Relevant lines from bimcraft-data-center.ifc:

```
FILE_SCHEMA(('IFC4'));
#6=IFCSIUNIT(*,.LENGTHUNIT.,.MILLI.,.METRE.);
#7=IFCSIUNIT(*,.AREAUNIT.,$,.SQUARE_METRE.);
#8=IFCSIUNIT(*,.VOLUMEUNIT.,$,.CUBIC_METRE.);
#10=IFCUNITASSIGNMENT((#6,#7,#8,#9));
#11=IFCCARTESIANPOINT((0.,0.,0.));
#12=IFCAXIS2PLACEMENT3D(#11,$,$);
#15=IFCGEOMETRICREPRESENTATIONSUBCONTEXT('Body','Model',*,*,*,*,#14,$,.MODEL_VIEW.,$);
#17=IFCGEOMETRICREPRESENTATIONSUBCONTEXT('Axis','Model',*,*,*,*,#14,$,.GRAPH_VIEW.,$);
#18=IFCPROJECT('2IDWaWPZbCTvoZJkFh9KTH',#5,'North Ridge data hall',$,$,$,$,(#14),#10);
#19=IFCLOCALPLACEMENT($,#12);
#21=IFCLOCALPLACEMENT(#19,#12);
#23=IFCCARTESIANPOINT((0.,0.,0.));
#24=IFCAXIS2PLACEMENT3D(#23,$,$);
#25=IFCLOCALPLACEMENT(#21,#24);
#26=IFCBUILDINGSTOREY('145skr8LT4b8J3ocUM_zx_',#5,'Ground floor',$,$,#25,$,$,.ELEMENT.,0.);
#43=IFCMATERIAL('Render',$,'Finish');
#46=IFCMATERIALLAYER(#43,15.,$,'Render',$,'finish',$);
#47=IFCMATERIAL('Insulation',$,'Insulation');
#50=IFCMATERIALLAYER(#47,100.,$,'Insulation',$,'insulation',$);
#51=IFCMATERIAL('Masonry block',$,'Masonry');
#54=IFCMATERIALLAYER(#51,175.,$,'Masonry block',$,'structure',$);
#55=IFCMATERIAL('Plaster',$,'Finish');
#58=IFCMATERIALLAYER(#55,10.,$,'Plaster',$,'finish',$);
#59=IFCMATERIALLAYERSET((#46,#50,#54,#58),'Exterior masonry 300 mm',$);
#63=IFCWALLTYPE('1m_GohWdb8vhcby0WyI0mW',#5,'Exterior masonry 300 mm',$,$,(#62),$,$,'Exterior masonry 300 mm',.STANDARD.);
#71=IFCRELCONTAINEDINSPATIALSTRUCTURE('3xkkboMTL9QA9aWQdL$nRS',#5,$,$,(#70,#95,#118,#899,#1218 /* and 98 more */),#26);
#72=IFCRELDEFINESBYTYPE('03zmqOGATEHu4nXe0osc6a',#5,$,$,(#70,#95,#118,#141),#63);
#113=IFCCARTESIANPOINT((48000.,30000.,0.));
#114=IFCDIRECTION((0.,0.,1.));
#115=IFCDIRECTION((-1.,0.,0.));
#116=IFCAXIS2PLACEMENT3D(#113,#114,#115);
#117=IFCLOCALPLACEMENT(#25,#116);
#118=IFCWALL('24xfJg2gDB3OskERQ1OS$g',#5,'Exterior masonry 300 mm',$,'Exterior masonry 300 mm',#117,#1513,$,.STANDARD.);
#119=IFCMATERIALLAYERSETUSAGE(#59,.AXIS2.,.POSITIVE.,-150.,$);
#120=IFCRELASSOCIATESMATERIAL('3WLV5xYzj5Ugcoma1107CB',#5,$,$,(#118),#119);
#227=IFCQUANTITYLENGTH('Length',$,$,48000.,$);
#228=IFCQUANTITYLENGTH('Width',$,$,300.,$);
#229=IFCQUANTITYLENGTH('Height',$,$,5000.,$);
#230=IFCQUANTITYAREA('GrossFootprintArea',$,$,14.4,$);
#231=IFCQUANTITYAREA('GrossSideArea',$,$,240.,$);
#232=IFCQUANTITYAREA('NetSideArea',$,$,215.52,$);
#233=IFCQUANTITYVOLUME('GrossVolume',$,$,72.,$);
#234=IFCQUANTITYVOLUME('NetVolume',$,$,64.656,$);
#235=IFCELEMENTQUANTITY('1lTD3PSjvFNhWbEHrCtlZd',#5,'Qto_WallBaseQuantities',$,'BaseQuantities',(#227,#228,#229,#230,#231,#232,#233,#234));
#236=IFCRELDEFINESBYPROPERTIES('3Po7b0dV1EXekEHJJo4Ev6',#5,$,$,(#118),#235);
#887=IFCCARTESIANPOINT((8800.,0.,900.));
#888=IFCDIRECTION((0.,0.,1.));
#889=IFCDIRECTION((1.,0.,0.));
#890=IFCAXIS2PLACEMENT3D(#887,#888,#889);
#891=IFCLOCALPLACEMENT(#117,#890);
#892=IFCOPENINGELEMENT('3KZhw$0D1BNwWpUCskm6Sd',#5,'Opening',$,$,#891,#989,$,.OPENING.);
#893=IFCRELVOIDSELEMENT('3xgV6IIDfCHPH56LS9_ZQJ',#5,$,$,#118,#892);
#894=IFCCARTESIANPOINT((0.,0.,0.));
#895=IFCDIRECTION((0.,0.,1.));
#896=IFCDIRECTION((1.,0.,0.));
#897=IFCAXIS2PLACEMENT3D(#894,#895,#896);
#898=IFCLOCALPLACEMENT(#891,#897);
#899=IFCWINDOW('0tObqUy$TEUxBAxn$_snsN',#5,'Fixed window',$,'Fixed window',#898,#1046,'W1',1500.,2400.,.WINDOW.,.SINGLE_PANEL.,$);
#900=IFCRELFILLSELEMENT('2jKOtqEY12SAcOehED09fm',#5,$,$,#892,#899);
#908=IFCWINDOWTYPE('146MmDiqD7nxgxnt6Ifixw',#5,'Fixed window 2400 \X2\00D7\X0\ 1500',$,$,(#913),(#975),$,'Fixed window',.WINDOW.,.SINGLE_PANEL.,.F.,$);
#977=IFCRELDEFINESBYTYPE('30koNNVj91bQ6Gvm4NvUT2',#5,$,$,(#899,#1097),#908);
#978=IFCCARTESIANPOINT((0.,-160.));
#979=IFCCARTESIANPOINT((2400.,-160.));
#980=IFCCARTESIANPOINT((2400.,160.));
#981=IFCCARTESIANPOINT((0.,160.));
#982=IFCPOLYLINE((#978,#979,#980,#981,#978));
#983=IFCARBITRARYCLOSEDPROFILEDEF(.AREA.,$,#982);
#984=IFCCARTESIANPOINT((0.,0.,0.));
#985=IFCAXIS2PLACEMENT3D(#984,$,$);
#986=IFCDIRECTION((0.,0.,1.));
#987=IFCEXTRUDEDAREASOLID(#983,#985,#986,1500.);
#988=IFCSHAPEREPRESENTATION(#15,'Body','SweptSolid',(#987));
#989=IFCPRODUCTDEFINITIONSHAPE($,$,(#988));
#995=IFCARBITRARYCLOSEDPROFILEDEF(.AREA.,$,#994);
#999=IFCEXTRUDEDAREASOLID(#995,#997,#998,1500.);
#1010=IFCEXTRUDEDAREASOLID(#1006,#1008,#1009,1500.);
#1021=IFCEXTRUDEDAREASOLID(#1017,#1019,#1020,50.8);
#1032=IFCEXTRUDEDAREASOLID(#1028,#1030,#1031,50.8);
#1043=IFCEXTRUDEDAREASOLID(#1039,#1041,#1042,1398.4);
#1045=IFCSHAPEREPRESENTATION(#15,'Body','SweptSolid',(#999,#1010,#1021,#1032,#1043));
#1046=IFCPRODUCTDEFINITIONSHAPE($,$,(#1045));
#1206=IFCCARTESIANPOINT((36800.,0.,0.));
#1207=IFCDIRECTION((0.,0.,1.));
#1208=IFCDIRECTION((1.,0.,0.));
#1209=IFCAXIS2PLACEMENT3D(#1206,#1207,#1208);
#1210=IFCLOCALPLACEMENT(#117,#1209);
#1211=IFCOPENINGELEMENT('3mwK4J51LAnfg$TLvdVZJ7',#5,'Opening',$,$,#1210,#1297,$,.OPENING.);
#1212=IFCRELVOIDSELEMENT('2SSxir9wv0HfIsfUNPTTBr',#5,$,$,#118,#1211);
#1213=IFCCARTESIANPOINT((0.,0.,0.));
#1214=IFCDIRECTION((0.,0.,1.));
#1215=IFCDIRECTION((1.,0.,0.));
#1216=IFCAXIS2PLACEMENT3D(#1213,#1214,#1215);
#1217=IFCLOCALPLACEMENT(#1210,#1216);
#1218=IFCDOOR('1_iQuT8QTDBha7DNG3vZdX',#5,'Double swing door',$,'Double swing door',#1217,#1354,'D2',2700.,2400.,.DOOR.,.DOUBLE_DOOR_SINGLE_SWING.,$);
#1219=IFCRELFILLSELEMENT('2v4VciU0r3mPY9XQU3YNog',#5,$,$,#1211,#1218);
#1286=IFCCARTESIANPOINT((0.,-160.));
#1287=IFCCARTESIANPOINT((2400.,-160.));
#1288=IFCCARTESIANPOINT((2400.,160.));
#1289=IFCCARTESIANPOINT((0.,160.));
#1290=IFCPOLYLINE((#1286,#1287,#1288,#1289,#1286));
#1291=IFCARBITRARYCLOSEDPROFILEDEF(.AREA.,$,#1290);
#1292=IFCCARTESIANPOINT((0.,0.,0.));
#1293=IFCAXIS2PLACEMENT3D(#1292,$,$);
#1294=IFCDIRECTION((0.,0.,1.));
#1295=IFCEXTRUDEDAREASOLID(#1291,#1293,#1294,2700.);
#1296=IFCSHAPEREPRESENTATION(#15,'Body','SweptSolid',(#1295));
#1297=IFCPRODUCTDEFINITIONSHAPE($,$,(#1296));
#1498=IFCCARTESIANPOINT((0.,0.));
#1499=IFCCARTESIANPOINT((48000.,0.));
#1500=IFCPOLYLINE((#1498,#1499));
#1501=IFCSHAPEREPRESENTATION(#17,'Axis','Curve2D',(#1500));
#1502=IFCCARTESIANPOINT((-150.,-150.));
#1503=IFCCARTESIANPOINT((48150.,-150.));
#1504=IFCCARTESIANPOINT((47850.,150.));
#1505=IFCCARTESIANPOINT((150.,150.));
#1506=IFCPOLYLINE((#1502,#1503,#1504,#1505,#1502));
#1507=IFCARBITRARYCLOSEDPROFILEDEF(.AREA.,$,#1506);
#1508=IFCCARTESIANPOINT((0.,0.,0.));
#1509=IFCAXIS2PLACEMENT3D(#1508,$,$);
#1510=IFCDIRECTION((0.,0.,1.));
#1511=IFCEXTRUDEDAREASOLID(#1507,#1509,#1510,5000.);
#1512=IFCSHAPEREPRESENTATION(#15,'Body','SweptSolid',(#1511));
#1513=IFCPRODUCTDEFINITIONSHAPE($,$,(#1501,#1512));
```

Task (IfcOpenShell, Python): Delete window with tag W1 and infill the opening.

```python
import ifcopenshell
import ifcopenshell.api.feature
import ifcopenshell.api.pset
import ifcopenshell.api.root
import ifcopenshell.geom
import ifcopenshell.util.element
import ifcopenshell.util.shape
import ifcopenshell.util.unit

model = ifcopenshell.open("bimcraft-data-center.ifc")
area_scale = ifcopenshell.util.unit.calculate_unit_scale(model, "AREAUNIT")
volume_scale = ifcopenshell.util.unit.calculate_unit_scale(model, "VOLUMEUNIT")
settings = ifcopenshell.geom.settings()


def volume(element):
    """Net volume in cubic metres, openings subtracted."""
    shape = ifcopenshell.geom.create_shape(settings, element)
    return ifcopenshell.util.shape.get_volume(shape.geometry)


window = model.by_id(899)
opening = window.FillsVoids[0].RelatingOpeningElement
wall = opening.VoidsElements[0].RelatingBuildingElement
before = volume(wall)

ifcopenshell.api.root.remove_product(model, product=window)
ifcopenshell.api.feature.remove_feature(model, feature=opening)

after = volume(wall)
thickness = 0.3  # wall thickness in metres

# Update the wall's stored quantities.
qto = model.by_id(ifcopenshell.util.element.get_pset(wall, "Qto_WallBaseQuantities", should_inherit=False)["id"])
ifcopenshell.api.pset.edit_qto(model, qto=qto, properties={
    "NetSideArea": after / thickness / area_scale,
    "NetVolume": after / volume_scale,
})

print(f"wall volume {before:.3f} -> {after:.3f} m3")

model.write("bimcraft-data-center_rev.ifc")
```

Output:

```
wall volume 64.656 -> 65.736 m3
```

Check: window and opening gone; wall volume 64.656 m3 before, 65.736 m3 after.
